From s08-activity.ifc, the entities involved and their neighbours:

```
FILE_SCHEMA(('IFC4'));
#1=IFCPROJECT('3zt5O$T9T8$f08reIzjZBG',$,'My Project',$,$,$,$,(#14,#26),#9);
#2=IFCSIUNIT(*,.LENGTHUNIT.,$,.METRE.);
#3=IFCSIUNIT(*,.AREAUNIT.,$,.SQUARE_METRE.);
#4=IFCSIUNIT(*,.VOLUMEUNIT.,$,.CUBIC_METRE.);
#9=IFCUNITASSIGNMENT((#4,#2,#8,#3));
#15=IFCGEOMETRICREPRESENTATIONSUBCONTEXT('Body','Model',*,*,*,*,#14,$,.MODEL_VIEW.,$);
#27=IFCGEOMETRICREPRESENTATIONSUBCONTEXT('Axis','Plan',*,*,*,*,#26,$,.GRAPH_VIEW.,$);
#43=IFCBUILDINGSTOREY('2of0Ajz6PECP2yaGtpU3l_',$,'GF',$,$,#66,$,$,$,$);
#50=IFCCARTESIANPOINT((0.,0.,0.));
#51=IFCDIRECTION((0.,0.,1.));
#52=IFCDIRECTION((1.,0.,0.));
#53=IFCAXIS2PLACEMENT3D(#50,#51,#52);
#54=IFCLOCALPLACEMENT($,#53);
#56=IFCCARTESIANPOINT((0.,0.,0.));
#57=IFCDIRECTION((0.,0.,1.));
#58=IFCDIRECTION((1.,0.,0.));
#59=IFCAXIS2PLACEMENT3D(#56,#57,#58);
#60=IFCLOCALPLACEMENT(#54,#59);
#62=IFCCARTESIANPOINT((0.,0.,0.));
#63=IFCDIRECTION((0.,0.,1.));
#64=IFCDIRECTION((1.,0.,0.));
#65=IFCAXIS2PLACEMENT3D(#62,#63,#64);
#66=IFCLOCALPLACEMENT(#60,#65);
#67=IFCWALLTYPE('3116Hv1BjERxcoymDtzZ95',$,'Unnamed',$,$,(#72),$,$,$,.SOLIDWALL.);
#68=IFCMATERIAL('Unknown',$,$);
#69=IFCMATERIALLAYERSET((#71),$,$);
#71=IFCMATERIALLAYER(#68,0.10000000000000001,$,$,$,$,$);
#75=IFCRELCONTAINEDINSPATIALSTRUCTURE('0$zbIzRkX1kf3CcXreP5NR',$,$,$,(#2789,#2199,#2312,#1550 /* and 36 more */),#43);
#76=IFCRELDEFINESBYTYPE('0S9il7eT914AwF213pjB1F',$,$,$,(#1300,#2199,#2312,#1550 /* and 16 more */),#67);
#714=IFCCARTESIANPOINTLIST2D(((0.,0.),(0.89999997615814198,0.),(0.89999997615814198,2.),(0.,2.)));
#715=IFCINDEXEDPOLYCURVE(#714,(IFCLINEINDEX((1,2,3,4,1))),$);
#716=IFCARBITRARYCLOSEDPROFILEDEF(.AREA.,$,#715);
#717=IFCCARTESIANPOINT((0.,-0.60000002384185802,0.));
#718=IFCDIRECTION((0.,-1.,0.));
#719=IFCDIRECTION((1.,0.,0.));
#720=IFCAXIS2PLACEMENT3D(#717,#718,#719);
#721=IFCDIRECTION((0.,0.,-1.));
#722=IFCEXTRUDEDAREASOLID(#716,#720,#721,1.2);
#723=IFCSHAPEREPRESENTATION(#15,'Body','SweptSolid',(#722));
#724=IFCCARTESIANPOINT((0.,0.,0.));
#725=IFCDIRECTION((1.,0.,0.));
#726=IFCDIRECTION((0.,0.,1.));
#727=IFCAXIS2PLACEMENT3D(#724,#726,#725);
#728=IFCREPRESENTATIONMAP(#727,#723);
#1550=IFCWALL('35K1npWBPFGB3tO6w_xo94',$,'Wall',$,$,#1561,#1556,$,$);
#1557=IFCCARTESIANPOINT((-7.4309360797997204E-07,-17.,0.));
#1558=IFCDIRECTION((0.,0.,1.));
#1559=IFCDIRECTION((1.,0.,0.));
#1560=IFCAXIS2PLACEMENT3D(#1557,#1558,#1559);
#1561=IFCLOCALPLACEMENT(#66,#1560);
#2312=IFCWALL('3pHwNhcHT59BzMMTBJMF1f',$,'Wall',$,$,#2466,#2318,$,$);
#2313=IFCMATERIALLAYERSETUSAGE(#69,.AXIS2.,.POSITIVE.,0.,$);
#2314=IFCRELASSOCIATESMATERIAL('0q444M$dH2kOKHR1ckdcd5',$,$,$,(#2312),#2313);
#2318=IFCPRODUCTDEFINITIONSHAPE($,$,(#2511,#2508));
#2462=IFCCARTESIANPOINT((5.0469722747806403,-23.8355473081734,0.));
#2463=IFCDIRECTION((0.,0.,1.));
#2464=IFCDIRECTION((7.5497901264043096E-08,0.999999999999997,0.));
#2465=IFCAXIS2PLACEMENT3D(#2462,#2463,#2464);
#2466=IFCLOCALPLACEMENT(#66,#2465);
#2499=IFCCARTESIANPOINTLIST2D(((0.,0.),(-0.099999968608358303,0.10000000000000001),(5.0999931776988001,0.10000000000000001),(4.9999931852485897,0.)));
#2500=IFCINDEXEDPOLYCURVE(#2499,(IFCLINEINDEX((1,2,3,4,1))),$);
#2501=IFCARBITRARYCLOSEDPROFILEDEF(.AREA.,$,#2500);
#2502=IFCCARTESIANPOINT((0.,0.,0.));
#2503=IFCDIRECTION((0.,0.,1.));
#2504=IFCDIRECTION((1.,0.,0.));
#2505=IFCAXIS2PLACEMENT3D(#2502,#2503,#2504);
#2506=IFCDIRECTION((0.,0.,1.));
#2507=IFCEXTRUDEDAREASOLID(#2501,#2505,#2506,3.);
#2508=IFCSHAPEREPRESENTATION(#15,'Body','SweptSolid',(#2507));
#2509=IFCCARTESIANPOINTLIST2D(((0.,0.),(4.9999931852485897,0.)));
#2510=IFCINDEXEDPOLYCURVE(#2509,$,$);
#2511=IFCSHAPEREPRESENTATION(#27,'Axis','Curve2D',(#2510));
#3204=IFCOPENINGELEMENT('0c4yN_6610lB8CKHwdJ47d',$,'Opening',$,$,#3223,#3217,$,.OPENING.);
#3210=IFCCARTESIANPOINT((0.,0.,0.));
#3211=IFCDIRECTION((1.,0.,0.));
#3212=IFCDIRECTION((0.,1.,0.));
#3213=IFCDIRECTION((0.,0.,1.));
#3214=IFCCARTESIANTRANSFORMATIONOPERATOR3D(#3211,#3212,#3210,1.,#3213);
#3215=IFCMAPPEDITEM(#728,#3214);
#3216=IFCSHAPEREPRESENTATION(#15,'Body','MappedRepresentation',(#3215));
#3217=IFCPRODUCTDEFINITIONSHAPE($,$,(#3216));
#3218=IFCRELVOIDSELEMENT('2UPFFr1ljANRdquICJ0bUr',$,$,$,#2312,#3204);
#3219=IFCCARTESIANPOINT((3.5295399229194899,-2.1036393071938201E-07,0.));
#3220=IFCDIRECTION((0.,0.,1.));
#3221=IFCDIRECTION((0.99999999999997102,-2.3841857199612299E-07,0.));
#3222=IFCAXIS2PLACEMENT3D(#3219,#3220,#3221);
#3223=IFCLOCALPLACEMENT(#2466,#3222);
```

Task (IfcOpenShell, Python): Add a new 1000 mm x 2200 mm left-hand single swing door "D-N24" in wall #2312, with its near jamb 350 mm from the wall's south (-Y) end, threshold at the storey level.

```python
import numpy as np
import ifcopenshell
import ifcopenshell.api.feature
import ifcopenshell.api.geometry
import ifcopenshell.api.root
import ifcopenshell.api.spatial
import ifcopenshell.geom
import ifcopenshell.util.element
import ifcopenshell.util.placement
import ifcopenshell.util.representation
import ifcopenshell.util.shape
import ifcopenshell.util.unit

model = ifcopenshell.open("s08-activity.ifc")
unit_scale = ifcopenshell.util.unit.calculate_unit_scale(model)
settings = ifcopenshell.geom.settings()


def volume(element):
    """Net volume in cubic metres, openings subtracted."""
    shape = ifcopenshell.geom.create_shape(settings, element)
    return ifcopenshell.util.shape.get_volume(shape.geometry)


wall = model.by_id(2312)
storey = ifcopenshell.util.element.get_container(wall, ifc_class="IfcBuildingStorey")
context = ifcopenshell.util.representation.get_context(model, "Model", "Body", "MODEL_VIEW")
before = volume(wall)

width, height, from_end, sill = 1, 2.2, 0.35, 0.0  # metres

# The wall runs along its own X axis, and the end named is its -X end.
wall_shape = ifcopenshell.geom.create_shape(settings, wall)
x, y, z = ifcopenshell.util.shape.get_vertices(wall_shape.geometry).T
start = x.min() + from_end
face, thickness = float(y.min()), float(y.max() - y.min())
wall_matrix = ifcopenshell.util.placement.get_local_placement(wall.ObjectPlacement)
level = ifcopenshell.util.placement.get_local_placement(storey.ObjectPlacement)[2, 3]


def in_wall(x, y):
    """Placement at x, y metres in the wall's axes, at sill height."""
    matrix = wall_matrix.copy()
    matrix[:, 3] = wall_matrix @ np.array([x / unit_scale, y / unit_scale, 0.0, 1.0])
    matrix[2, 3] = level + sill / unit_scale
    return matrix


# Opening: a box that overshoots both wall faces by 50 mm.
opening = ifcopenshell.api.root.create_entity(model, ifc_class="IfcOpeningElement", predefined_type="OPENING")
box = ifcopenshell.api.geometry.add_wall_representation(
    model, context=context, length=width, height=height, thickness=thickness + 0.1
)
ifcopenshell.api.geometry.assign_representation(model, product=opening, representation=box)
ifcopenshell.api.geometry.edit_object_placement(model, product=opening, matrix=in_wall(start, face - 0.05), is_si=False)
ifcopenshell.api.feature.add_feature(model, feature=opening, element=wall)

door = ifcopenshell.api.root.create_entity(model, ifc_class="IfcDoor", name="D-N24", predefined_type="DOOR")
door.OverallWidth, door.OverallHeight = width / unit_scale, height / unit_scale
door.OperationType = "SINGLE_SWING_LEFT"
body = ifcopenshell.api.geometry.add_door_representation(
    model,
    context=context,
    overall_width=door.OverallWidth,
    overall_height=door.OverallHeight,
    operation_type="SINGLE_SWING_LEFT",
    lining_properties={"LiningDepth": thickness / unit_scale, "ThresholdDepth": thickness / unit_scale},
)
ifcopenshell.api.geometry.assign_representation(model, product=door, representation=body)
ifcopenshell.api.spatial.assign_container(model, products=[door], relating_structure=storey)
ifcopenshell.api.feature.add_filling(model, opening=opening, element=door)

# The lining spans the wall, so the door starts at the wall face.
ifcopenshell.api.geometry.edit_object_placement(model, product=door, matrix=in_wall(start, face), is_si=False)

after = volume(wall)

print(f"wall volume {before:.3f} -> {after:.3f} m3")

model.write("s08-activity_v2.ifc")
```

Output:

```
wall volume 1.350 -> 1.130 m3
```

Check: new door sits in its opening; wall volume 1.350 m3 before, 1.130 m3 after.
